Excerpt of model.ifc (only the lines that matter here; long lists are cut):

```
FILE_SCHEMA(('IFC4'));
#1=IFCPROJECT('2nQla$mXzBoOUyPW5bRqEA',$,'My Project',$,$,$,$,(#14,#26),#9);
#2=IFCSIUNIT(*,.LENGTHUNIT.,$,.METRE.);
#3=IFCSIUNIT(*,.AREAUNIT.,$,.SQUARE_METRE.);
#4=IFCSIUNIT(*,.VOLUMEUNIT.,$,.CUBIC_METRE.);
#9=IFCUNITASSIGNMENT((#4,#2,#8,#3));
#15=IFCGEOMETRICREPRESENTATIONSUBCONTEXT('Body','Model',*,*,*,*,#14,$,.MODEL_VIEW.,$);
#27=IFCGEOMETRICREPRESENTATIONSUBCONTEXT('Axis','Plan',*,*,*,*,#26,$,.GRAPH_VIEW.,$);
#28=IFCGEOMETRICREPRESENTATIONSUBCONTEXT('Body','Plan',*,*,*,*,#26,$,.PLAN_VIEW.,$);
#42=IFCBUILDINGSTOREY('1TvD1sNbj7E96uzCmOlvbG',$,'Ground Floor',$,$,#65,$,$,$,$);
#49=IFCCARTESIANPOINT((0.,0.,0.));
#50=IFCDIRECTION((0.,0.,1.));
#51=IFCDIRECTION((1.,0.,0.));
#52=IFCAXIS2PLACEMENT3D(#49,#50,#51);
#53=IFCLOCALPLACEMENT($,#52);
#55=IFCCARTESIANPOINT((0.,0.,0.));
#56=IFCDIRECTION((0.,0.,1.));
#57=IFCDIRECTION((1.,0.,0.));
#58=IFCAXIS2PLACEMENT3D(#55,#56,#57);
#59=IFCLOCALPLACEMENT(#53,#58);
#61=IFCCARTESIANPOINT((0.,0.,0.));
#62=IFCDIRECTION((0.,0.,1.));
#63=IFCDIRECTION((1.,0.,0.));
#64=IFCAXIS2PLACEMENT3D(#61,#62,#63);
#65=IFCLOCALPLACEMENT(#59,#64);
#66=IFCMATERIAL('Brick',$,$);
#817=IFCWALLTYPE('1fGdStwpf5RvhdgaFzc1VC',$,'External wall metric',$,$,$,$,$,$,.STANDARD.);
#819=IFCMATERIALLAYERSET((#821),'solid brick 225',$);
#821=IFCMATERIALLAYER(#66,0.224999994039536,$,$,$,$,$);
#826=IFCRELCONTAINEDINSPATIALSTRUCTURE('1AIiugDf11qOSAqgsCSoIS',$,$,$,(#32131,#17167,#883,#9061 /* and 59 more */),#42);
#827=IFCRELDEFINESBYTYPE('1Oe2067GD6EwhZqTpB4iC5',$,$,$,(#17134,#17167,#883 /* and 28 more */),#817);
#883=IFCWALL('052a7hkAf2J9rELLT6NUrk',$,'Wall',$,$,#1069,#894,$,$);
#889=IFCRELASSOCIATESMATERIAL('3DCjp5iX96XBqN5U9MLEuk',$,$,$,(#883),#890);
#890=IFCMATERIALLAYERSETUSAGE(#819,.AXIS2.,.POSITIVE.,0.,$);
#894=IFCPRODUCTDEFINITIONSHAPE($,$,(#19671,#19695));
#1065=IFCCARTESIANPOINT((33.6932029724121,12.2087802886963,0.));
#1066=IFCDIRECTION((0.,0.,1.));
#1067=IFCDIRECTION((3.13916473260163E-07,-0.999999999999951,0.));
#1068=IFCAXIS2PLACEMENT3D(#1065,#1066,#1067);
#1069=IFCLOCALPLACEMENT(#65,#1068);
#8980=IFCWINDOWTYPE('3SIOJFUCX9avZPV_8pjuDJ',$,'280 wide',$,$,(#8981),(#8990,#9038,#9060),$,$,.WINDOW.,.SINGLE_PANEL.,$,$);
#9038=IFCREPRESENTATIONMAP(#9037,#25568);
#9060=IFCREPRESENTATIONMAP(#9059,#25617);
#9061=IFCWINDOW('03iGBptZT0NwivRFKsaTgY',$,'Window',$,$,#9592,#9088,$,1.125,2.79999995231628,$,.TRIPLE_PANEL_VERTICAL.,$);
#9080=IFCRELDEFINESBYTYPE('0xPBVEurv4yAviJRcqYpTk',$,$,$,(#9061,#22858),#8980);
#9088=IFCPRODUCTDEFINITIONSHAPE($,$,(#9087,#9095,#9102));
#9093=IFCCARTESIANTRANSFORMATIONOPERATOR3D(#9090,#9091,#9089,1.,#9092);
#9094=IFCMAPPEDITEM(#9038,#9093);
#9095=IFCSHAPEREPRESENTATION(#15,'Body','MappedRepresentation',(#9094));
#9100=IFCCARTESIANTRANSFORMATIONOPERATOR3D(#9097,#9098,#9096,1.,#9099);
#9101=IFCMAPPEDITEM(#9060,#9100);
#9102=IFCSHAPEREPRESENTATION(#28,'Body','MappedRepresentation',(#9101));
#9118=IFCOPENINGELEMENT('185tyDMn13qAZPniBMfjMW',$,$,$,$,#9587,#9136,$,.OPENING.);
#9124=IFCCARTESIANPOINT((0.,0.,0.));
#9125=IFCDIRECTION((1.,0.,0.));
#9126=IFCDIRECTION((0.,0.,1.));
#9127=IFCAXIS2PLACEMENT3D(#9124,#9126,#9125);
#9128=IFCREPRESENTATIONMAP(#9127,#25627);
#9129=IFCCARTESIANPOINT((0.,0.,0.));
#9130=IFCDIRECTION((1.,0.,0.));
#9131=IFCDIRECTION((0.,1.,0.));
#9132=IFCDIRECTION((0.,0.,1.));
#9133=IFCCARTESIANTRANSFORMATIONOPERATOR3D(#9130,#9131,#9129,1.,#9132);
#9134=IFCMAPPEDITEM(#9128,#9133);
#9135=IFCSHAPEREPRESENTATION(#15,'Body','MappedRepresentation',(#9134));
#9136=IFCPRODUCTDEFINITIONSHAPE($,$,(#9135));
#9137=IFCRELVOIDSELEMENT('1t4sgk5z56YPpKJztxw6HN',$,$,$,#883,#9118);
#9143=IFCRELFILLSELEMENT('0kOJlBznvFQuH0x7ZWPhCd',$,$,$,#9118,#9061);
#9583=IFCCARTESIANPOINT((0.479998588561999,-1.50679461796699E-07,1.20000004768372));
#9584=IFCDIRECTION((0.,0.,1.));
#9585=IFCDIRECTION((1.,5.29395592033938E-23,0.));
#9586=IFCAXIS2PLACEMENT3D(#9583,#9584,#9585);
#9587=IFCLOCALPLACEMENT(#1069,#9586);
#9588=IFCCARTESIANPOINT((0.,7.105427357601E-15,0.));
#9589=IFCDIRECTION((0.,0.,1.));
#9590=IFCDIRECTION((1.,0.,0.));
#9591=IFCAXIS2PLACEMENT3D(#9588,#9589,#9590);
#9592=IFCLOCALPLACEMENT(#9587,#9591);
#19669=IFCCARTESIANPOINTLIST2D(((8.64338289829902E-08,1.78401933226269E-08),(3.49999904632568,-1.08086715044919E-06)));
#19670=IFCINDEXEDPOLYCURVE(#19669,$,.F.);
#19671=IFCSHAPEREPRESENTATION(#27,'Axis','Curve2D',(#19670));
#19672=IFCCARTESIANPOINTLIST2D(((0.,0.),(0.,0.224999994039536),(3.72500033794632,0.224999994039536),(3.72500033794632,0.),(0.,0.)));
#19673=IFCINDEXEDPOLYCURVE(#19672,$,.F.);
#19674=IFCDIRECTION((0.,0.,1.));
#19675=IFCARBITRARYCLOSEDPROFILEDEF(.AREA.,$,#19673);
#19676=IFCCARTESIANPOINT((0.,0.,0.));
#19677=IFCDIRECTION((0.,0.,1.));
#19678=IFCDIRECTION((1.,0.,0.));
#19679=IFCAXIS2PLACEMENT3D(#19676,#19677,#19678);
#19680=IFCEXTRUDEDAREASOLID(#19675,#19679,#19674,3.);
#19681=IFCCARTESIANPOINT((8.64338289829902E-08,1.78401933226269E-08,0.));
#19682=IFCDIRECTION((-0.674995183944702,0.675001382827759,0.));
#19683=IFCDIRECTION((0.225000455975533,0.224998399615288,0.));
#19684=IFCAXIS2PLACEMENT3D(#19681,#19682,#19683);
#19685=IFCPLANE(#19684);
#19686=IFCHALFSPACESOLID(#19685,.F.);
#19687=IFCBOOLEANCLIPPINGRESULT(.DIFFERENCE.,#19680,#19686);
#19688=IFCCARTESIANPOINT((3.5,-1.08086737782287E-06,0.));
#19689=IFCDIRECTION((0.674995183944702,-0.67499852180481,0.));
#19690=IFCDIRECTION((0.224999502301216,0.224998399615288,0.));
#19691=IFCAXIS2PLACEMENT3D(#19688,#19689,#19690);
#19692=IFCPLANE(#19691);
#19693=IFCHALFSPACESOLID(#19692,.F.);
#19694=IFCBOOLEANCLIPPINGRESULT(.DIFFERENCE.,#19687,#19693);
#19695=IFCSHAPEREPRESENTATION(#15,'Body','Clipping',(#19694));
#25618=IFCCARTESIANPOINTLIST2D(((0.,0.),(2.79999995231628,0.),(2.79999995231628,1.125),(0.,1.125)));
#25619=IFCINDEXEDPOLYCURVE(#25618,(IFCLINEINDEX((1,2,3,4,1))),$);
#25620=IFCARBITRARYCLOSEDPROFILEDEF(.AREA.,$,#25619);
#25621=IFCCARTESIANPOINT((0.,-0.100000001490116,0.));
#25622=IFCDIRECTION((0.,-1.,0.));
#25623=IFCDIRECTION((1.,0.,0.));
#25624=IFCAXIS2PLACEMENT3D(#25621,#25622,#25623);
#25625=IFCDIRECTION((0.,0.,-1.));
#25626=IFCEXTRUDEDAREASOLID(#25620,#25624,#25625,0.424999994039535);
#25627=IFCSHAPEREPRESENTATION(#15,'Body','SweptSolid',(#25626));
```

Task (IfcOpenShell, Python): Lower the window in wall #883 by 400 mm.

```python
import numpy as np
import ifcopenshell
import ifcopenshell.api.geometry
import ifcopenshell.util.placement
import ifcopenshell.util.unit

model = ifcopenshell.open("model.ifc")
unit_scale = ifcopenshell.util.unit.calculate_unit_scale(model)

window = model.by_id(9061)
opening = window.FillsVoids[0].RelatingOpeningElement
dz = -0.4 / unit_scale

shift = np.array([0.0, 0.0, dz])
# The window is placed relative to its opening, so it follows when the opening moves.
matrix = ifcopenshell.util.placement.get_local_placement(opening.ObjectPlacement)
matrix[:3, 3] += shift
ifcopenshell.api.geometry.edit_object_placement(
    model, product=opening, matrix=matrix, is_si=False, should_transform_children=True
)

print(f"moved by {dz * unit_scale:+.3f} m")

model.write("model_rev.ifc")
```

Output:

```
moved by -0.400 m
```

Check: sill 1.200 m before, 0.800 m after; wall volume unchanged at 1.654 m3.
